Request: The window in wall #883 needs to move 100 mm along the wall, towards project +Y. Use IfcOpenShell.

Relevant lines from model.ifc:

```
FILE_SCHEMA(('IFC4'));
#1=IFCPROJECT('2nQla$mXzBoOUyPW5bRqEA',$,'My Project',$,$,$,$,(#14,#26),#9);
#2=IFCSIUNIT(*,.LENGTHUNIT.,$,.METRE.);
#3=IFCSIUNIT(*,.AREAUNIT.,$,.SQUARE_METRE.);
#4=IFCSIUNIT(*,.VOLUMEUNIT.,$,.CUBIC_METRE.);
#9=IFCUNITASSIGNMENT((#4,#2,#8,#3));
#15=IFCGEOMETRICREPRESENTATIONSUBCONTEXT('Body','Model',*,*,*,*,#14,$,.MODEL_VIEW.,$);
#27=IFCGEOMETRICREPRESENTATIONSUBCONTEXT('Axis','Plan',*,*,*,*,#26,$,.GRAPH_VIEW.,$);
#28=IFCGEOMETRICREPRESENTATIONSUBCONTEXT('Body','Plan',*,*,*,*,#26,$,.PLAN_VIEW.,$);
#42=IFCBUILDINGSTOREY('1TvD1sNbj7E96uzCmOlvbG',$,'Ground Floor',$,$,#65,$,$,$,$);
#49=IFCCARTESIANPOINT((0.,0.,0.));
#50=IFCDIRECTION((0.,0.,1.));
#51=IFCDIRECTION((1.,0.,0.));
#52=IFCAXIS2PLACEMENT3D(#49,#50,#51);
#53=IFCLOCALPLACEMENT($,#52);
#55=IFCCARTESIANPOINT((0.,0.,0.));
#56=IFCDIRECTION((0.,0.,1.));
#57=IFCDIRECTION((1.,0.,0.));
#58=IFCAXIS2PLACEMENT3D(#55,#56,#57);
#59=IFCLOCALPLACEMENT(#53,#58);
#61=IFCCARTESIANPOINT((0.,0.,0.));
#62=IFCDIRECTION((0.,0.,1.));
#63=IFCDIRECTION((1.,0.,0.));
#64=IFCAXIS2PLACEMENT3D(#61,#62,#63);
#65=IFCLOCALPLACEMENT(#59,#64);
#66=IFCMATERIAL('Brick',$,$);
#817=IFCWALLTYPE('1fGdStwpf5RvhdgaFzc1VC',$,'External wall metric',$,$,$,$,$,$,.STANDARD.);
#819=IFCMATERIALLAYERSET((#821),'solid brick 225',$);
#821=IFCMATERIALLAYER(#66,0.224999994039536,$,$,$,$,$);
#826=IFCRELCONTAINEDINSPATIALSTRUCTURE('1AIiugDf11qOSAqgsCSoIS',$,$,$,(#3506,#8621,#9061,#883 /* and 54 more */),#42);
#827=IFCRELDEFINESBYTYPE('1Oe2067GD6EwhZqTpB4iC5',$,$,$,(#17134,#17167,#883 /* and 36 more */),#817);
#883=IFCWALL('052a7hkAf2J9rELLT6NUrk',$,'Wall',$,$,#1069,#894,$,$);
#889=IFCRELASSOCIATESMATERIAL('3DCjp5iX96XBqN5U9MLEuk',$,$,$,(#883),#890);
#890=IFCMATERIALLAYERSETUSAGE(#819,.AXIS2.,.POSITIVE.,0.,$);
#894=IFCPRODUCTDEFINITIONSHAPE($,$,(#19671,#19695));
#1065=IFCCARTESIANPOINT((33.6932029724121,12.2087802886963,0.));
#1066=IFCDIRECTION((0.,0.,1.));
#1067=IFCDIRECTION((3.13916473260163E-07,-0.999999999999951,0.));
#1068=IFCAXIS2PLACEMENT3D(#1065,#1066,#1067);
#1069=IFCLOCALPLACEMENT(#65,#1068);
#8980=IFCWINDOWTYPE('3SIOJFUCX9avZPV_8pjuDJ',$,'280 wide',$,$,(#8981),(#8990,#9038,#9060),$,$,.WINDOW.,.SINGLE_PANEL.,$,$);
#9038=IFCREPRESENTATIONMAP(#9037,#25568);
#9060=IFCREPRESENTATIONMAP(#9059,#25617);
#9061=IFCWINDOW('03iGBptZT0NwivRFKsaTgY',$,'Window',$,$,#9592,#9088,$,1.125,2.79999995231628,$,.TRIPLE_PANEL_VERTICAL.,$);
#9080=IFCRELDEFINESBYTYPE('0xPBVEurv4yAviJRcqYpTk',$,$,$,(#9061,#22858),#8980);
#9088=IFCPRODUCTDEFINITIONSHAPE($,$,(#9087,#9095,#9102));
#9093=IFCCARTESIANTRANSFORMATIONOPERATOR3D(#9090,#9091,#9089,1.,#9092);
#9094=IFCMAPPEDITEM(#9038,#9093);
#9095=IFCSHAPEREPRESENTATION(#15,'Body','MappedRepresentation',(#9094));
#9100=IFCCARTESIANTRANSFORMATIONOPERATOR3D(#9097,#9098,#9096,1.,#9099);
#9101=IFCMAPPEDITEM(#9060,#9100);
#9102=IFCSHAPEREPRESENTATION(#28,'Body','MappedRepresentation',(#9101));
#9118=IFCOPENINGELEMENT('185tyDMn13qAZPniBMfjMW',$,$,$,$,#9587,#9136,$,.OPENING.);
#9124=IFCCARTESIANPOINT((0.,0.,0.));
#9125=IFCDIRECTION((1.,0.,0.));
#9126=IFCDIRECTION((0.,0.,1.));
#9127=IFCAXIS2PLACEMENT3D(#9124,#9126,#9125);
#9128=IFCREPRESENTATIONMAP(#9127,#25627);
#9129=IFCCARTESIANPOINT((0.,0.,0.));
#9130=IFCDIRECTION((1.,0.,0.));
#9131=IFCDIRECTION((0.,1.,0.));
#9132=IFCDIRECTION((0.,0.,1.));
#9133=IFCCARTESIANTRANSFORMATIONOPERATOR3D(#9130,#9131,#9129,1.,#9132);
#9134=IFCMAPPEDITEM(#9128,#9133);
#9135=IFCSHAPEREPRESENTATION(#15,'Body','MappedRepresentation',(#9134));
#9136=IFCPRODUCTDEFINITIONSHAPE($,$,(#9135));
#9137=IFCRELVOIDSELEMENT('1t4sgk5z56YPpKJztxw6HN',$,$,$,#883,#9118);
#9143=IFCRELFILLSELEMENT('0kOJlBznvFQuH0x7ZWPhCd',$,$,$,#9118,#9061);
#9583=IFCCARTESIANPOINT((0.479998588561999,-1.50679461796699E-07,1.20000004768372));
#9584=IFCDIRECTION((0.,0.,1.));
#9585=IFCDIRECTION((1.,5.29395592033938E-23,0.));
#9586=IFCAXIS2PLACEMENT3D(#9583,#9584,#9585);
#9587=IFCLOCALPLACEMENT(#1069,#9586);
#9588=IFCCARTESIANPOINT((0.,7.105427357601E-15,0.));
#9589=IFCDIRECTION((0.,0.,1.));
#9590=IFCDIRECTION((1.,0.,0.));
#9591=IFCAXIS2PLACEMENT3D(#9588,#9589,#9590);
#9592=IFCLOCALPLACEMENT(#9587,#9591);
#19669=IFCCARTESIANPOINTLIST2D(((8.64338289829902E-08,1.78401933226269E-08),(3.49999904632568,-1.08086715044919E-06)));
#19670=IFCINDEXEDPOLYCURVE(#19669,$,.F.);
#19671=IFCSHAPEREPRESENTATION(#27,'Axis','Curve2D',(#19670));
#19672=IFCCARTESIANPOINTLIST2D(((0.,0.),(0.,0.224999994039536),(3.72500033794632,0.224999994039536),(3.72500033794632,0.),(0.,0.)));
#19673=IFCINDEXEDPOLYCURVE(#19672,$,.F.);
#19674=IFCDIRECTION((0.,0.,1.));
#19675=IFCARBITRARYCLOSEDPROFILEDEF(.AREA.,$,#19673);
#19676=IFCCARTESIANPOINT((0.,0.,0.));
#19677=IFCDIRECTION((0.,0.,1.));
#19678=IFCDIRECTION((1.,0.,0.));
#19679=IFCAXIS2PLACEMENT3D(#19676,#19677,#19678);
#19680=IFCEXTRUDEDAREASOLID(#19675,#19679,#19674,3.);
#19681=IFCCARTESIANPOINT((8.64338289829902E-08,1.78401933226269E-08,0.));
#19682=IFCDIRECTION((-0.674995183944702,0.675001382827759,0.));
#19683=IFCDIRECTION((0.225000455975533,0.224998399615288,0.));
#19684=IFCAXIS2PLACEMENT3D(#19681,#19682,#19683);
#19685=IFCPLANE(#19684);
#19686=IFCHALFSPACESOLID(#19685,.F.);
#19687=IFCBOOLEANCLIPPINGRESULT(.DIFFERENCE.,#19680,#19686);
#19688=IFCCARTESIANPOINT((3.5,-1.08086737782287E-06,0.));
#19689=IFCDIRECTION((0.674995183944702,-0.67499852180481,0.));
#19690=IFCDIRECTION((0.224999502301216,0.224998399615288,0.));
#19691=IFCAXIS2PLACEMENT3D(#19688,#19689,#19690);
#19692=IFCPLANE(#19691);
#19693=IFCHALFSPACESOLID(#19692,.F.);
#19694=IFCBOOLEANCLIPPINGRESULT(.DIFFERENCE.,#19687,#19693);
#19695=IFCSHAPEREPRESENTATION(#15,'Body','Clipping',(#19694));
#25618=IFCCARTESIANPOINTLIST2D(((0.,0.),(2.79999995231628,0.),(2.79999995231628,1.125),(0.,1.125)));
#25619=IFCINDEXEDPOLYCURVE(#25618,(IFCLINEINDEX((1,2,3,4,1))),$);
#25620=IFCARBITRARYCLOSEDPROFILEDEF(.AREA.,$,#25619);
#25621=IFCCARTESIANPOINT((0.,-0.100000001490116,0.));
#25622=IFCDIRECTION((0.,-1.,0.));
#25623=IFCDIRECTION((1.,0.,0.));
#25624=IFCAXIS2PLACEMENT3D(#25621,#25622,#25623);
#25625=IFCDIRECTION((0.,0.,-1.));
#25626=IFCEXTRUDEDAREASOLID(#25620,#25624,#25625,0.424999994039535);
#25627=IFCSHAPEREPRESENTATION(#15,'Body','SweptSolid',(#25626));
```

```python
import ifcopenshell
import ifcopenshell.api.geometry
import ifcopenshell.util.placement
import ifcopenshell.util.unit

model = ifcopenshell.open("model.ifc")
unit_scale = ifcopenshell.util.unit.calculate_unit_scale(model)

window = model.by_guid("03iGBptZT0NwivRFKsaTgY")
opening = window.FillsVoids[0].RelatingOpeningElement
wall = opening.VoidsElements[0].RelatingBuildingElement

wall_matrix = ifcopenshell.util.placement.get_local_placement(wall.ObjectPlacement)
shift = wall_matrix[:3, 0] * -0.1 / unit_scale
before = ifcopenshell.util.placement.get_local_placement(window.ObjectPlacement)[:3, 3].copy()

# The window is placed relative to its opening, so it follows when the opening moves.
matrix = ifcopenshell.util.placement.get_local_placement(opening.ObjectPlacement)
matrix[:3, 3] += shift
ifcopenshell.api.geometry.edit_object_placement(
    model, product=opening, matrix=matrix, is_si=False, should_transform_children=True
)

after = ifcopenshell.util.placement.get_local_placement(window.ObjectPlacement)[:3, 3]
print("window moved by", (after - before).round(3) + 0.0)

model.write("model_rev.ifc")
```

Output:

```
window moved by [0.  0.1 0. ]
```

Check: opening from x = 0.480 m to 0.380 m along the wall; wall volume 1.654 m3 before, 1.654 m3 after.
